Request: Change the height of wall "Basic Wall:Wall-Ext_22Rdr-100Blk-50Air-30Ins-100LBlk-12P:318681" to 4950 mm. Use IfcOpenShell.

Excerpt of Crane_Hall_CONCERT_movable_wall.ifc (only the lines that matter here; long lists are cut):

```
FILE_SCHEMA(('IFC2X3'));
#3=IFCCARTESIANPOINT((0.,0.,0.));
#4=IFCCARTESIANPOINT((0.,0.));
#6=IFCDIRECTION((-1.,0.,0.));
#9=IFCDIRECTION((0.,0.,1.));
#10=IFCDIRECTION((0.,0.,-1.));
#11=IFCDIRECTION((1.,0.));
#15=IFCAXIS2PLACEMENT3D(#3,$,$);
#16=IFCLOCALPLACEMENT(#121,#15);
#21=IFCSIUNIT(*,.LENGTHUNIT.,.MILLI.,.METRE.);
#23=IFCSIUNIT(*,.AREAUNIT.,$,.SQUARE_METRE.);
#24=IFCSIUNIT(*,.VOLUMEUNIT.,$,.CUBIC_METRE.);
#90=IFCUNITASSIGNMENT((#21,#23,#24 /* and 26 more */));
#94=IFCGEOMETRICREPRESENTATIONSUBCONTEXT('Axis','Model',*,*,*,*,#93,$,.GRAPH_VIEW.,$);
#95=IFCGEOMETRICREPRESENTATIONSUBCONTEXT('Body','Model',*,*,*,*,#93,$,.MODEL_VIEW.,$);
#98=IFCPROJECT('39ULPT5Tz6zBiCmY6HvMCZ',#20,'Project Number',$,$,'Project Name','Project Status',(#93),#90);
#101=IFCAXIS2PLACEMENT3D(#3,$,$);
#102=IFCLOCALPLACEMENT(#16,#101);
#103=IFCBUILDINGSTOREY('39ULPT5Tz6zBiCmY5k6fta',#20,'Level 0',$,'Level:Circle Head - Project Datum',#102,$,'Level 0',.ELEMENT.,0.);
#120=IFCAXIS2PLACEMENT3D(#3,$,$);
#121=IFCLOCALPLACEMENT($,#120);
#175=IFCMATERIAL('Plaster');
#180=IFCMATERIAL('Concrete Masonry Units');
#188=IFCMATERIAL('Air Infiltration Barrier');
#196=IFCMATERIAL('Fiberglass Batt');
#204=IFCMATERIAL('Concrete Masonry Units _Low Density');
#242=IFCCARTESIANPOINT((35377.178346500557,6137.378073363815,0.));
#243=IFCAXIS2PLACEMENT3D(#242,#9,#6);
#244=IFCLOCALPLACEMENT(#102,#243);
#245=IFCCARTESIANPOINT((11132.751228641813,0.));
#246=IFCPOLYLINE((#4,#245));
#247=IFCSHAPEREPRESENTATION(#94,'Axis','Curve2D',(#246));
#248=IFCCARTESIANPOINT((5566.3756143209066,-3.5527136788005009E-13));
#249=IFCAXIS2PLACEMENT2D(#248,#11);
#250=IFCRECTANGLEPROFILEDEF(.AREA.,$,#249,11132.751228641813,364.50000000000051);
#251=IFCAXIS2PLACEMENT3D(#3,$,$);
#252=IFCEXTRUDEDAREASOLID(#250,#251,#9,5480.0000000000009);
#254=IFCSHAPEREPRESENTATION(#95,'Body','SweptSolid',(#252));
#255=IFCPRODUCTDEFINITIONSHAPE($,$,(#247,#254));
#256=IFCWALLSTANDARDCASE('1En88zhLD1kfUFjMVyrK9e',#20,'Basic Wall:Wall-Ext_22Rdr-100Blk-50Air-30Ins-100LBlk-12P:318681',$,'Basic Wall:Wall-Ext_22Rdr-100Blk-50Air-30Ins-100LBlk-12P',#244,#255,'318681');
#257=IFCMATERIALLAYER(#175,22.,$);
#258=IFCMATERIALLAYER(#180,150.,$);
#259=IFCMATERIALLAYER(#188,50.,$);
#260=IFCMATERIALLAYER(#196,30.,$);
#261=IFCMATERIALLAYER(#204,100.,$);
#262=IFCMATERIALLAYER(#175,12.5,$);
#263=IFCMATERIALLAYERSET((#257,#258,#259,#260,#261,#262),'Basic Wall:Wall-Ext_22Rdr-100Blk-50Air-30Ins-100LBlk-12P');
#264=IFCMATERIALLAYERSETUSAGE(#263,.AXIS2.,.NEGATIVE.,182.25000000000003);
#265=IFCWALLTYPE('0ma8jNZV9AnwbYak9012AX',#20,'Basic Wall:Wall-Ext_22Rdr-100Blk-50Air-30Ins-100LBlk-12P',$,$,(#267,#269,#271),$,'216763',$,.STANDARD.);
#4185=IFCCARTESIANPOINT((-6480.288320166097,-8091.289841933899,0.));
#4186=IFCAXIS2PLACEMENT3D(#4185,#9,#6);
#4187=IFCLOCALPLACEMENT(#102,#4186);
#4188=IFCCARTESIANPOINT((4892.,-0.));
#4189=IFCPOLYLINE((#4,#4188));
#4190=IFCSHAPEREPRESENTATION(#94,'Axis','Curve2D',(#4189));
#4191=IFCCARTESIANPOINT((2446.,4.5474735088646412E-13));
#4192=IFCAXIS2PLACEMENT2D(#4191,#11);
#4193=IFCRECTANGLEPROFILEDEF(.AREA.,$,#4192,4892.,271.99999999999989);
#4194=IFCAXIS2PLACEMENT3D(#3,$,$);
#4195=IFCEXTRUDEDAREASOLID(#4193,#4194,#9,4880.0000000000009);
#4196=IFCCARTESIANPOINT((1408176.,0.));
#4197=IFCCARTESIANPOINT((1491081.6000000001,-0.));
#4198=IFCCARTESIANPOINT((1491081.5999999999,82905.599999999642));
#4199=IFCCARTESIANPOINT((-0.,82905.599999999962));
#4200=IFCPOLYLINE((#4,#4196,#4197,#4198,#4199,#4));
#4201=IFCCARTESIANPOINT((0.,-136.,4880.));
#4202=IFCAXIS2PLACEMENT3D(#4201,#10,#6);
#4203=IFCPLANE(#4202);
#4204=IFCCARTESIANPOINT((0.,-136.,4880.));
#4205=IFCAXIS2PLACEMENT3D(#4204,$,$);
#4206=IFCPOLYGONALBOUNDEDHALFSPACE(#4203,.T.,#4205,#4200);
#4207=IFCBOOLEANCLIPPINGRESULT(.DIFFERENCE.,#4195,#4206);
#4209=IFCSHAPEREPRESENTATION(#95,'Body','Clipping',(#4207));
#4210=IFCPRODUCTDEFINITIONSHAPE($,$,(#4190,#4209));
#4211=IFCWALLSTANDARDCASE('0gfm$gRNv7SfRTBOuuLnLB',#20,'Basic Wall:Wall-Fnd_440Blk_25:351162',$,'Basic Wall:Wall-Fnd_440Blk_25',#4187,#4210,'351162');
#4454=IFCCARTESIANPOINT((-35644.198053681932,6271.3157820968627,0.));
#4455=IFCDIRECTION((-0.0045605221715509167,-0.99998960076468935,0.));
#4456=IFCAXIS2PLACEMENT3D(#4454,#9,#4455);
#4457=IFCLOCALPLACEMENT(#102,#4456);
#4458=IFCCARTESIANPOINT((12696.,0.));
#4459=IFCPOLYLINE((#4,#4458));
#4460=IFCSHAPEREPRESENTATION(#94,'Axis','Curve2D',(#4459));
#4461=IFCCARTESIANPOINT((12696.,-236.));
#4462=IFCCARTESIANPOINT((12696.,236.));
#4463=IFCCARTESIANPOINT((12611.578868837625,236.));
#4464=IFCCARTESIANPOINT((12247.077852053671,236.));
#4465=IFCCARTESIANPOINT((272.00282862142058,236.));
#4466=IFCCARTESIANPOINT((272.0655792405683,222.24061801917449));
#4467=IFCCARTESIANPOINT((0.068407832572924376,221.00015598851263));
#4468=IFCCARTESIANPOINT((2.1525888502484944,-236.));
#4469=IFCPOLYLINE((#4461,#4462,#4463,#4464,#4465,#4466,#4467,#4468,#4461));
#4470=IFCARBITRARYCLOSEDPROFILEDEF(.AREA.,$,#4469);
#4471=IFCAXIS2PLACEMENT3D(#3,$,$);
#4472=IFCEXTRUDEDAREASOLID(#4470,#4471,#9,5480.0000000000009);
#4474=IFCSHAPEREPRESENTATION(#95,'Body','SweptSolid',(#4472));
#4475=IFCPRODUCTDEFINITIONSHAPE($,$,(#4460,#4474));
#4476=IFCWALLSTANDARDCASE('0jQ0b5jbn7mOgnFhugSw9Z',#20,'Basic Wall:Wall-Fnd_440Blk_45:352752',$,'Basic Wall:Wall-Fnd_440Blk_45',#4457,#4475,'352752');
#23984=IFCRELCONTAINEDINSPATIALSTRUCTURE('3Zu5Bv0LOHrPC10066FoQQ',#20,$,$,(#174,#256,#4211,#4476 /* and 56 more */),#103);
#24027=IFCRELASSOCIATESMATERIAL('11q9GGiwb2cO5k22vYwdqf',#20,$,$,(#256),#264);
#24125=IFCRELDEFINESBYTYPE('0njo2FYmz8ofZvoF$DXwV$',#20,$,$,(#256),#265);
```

```python
import ifcopenshell
import ifcopenshell.geom
import ifcopenshell.util.representation
import ifcopenshell.util.shape
import ifcopenshell.util.unit

model = ifcopenshell.open("Crane_Hall_CONCERT_movable_wall.ifc")
unit_scale = ifcopenshell.util.unit.calculate_unit_scale(model)
settings = ifcopenshell.geom.settings()


def volume(element):
    """Net volume in cubic metres, openings subtracted."""
    shape = ifcopenshell.geom.create_shape(settings, element)
    return ifcopenshell.util.shape.get_volume(shape.geometry)


wall = model.by_guid("1En88zhLD1kfUFjMVyrK9e")
before = volume(wall)

body = ifcopenshell.util.representation.get_representation(wall, "Model", "Body")
solid = body.Items[0]
old_height = solid.Depth
solid.Depth = 4.95 / unit_scale
after = volume(wall)

print(f"height {old_height:g} -> {solid.Depth:g}, volume {before:.3f} -> {after:.3f} m3")

model.write("Crane_Hall_CONCERT_movable_wall_v2.ifc")
```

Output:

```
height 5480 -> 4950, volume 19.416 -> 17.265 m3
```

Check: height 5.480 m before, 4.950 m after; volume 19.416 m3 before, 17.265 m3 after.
